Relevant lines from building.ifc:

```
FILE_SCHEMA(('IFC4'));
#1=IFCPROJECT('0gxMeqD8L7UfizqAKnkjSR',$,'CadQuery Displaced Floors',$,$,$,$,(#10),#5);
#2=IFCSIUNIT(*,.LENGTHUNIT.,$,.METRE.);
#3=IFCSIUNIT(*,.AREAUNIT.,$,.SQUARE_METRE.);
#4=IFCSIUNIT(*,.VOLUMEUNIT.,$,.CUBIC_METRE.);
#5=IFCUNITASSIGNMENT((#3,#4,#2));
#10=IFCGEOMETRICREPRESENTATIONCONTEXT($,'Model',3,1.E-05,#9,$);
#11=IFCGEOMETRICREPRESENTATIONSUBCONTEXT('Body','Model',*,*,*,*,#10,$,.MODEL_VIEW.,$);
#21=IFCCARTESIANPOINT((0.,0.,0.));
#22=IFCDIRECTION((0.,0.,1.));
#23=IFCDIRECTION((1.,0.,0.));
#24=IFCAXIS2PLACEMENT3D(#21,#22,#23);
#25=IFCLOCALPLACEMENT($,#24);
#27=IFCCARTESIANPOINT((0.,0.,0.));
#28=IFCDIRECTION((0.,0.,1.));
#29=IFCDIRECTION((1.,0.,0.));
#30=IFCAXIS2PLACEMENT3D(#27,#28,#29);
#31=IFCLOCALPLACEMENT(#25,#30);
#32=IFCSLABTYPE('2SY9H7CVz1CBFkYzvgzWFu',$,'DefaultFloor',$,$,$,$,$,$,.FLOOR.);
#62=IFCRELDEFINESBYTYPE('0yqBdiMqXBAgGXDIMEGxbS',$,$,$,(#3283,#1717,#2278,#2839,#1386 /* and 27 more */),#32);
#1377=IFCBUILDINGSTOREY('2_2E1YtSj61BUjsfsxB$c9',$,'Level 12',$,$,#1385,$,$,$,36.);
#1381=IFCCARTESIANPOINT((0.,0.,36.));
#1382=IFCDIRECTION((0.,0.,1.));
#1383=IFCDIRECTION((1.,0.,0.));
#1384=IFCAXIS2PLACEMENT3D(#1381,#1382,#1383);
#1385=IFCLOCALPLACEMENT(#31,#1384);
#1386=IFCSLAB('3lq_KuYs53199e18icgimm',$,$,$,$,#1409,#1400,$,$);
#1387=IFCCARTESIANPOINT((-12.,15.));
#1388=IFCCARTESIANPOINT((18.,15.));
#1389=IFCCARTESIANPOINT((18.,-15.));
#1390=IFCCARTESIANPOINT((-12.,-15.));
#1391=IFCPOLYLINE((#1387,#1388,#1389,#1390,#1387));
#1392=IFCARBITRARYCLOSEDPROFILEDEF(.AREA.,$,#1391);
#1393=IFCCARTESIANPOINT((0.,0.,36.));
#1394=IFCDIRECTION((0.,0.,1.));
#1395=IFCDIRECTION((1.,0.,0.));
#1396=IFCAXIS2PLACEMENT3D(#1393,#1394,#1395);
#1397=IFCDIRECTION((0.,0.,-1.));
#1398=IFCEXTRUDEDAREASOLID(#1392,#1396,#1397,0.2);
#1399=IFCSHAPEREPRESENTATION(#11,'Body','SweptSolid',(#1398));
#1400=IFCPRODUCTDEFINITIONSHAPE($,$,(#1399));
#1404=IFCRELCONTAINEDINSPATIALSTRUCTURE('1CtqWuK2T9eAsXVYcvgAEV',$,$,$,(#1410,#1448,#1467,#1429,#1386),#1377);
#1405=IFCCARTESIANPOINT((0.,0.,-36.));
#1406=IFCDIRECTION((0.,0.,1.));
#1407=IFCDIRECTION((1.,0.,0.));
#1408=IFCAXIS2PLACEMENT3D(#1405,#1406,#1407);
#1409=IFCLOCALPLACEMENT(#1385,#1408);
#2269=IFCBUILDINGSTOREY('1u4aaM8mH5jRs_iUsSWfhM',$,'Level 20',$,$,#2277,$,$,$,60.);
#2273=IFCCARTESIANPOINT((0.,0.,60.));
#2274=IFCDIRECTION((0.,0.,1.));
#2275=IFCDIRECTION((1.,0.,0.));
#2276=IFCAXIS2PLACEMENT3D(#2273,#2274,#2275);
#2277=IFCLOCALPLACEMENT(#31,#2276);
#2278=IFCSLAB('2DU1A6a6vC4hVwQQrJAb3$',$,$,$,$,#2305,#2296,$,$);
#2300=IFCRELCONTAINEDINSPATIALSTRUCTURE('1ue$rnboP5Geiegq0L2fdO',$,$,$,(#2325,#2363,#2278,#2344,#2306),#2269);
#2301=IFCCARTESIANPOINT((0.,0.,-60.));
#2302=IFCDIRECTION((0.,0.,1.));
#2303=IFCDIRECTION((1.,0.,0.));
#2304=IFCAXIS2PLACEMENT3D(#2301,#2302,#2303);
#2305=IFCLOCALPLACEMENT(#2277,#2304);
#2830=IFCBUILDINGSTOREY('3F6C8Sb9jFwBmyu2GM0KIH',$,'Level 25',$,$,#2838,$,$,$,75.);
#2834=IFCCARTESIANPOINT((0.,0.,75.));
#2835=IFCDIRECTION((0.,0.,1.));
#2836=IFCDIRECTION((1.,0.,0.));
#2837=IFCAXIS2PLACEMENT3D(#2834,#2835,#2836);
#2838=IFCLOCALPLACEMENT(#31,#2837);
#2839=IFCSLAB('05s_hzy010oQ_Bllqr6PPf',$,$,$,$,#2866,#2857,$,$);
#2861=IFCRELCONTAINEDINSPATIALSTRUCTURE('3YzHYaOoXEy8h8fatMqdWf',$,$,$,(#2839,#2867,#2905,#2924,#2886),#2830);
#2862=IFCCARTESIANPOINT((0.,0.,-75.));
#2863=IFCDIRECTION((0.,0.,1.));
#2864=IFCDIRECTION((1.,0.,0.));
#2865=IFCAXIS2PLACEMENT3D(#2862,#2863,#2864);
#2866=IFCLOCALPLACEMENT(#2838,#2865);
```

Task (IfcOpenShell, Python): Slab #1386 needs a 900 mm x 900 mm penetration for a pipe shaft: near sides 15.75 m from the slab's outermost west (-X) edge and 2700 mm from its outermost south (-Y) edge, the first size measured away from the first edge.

```python
import numpy as np
import ifcopenshell
import ifcopenshell.api.feature
import ifcopenshell.api.geometry
import ifcopenshell.api.root
import ifcopenshell.geom
import ifcopenshell.util.placement
import ifcopenshell.util.representation
import ifcopenshell.util.shape
import ifcopenshell.util.unit

model = ifcopenshell.open("building.ifc")
unit_scale = ifcopenshell.util.unit.calculate_unit_scale(model)
settings = ifcopenshell.geom.settings()


def volume(element):
    """Net volume in cubic metres, openings subtracted."""
    shape = ifcopenshell.geom.create_shape(settings, element)
    return ifcopenshell.util.shape.get_volume(shape.geometry)


slab = model.by_guid("3lq_KuYs53199e18icgimm")
before = volume(slab)

# Extent in the slab's own axes, in metres. The edges named are its -X and -Y sides.
slab_shape = ifcopenshell.geom.create_shape(settings, slab)
vertices = ifcopenshell.util.shape.get_vertices(slab_shape.geometry)
x_min, y_min, bottom = vertices.min(axis=0)
top = vertices[:, 2].max()

opening = ifcopenshell.api.root.create_entity(model, ifc_class="IfcOpeningElement", name="Pipe shaft opening", predefined_type="OPENING")
context = ifcopenshell.util.representation.get_context(model, "Model", "Body", "MODEL_VIEW")
width, depth = 0.9, 0.9
outline = [(0.0, 0.0), (width, 0.0), (width, depth), (0.0, depth), (0.0, 0.0)]
# Overshoot both faces by 50 mm so the cut is clean.
shape = ifcopenshell.api.geometry.add_slab_representation(
    model, context=context, depth=top - bottom + 0.1, polyline=outline
)
ifcopenshell.api.geometry.assign_representation(model, product=opening, representation=shape)

matrix = ifcopenshell.util.placement.get_local_placement(slab.ObjectPlacement)
matrix[:, 3] = matrix @ np.append(np.array([x_min + 15.75, y_min + 2.7, bottom - 0.05]) / unit_scale, 1.0)
ifcopenshell.api.geometry.edit_object_placement(model, product=opening, matrix=matrix, is_si=False)
ifcopenshell.api.feature.add_feature(model, feature=opening, element=slab)

after = volume(slab)

print(f"slab volume {before:.3f} -> {after:.3f} m3")

model.write("building_rev.ifc")
```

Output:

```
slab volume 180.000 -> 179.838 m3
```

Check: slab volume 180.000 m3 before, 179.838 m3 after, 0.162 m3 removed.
